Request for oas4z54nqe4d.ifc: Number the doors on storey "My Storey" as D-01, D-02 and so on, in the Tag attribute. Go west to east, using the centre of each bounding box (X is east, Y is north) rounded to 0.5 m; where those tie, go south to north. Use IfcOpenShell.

First a look at what the model holds.

```python
import ifcopenshell
import ifcopenshell.util.element
import ifcopenshell.util.placement

model = ifcopenshell.open("oas4z54nqe4d.ifc")
print(model.schema)
storey = next(s for s in model.by_type("IfcBuildingStorey") if s.Name == "My Storey")
doors = [e for e in ifcopenshell.util.element.get_decomposition(storey) if e.is_a("IfcDoor")]
for e in sorted(doors, key=lambda e: e.id()):
    origin = ifcopenshell.util.placement.get_local_placement(e.ObjectPlacement)[:3, 3]
    print(e.id(), e.Tag, e.Name, origin.round(2) + 0.0, sep=" | ")
```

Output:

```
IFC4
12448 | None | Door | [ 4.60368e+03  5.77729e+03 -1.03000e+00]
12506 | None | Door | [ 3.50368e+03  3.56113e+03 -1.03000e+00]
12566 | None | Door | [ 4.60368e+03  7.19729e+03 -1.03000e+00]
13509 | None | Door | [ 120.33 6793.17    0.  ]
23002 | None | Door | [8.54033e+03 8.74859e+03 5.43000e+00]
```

```python
import ifcopenshell
import ifcopenshell.geom
import ifcopenshell.util.element
import ifcopenshell.util.shape

model = ifcopenshell.open("oas4z54nqe4d.ifc")
settings = ifcopenshell.geom.settings()
settings.set("use-world-coords", True)


def centre(element):
    shape = ifcopenshell.geom.create_shape(settings, element)
    return ifcopenshell.util.shape.get_bbox_centroid(shape.geometry)


storey = next(s for s in model.by_type("IfcBuildingStorey") if s.Name == "My Storey")
doors = [e for e in ifcopenshell.util.element.get_decomposition(storey) if e.is_a("IfcDoor")]

# Insertion points can sit at a corner or the storey origin, so sort by the geometry (in metres).
centres = {e: centre(e) for e in doors}
doors.sort(key=lambda e: (round(centres[e][0] / 0.5), centres[e][1]))

for i, e in enumerate(doors, start=1):
    number = f"D-{i:02d}"
    e.Tag = number
    print(e.id(), number)

model.write("oas4z54nqe4d_edited.ifc")
```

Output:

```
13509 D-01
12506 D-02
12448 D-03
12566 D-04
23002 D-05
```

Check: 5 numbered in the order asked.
